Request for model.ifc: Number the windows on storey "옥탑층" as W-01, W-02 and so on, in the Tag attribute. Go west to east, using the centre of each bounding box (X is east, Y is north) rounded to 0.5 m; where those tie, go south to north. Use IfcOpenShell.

First a look at what the model holds.

```python
import ifcopenshell
import ifcopenshell.util.element
import ifcopenshell.util.placement

model = ifcopenshell.open("model.ifc")
print(model.schema)
storey = next(s for s in model.by_type("IfcBuildingStorey") if s.Name == "옥탑층")
windows = [e for e in ifcopenshell.util.element.get_decomposition(storey) if e.is_a("IfcWindow")]
for e in sorted(windows, key=lambda e: e.id()):
    origin = ifcopenshell.util.placement.get_local_placement(e.ObjectPlacement)[:3, 3]
    print(e.id(), e.Tag, e.Name, origin.round(2) + 0.0, sep=" | ")
```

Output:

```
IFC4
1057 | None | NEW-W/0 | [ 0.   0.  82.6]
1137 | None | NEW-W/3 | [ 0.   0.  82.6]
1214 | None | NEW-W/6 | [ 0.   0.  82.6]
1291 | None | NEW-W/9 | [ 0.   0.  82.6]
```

```python
import ifcopenshell
import ifcopenshell.geom
import ifcopenshell.util.element
import ifcopenshell.util.shape

model = ifcopenshell.open("model.ifc")
settings = ifcopenshell.geom.settings()
settings.set("use-world-coords", True)


def centre(element):
    shape = ifcopenshell.geom.create_shape(settings, element)
    return ifcopenshell.util.shape.get_bbox_centroid(shape.geometry)


storey = next(s for s in model.by_type("IfcBuildingStorey") if s.Name == "옥탑층")
windows = [e for e in ifcopenshell.util.element.get_decomposition(storey) if e.is_a("IfcWindow")]

# Insertion points can sit at a corner or the storey origin, so sort by the geometry (in metres).
centres = {e: centre(e) for e in windows}
windows.sort(key=lambda e: (round(centres[e][0] / 0.5), centres[e][1]))

for i, e in enumerate(windows, start=1):
    number = f"W-{i:02d}"
    e.Tag = number
    print(e.id(), number)

model.write("model_v2.ifc")
```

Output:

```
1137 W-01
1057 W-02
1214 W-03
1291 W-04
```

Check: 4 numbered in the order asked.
